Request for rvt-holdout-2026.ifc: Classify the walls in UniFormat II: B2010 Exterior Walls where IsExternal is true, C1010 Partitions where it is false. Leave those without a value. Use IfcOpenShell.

First a look at what the model holds.

```python
import ifcopenshell
import ifcopenshell.util.element

model = ifcopenshell.open("rvt-holdout-2026.ifc")
print(model.schema)
print("classifications:", [c.Name for c in model.by_type("IfcClassification")])
values = [ifcopenshell.util.element.get_pset(e, "Pset_WallCommon", "IsExternal") for e in model.by_type("IfcWall")]
for value in (True, False, None):
    print("IsExternal", value, values.count(value))
```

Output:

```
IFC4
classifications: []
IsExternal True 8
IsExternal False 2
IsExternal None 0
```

```python
import ifcopenshell
import ifcopenshell.api.classification
import ifcopenshell.util.element

model = ifcopenshell.open("rvt-holdout-2026.ifc")

system = ifcopenshell.api.classification.add_classification(model, classification="UniFormat II")

walls = model.by_type("IfcWall")
external = {e: ifcopenshell.util.element.get_pset(e, "Pset_WallCommon", "IsExternal") for e in walls}
for flag, code, name in ((True, "B2010", "Exterior Walls"), (False, "C1010", "Partitions")):
    products = [e for e in walls if external[e] is flag]
    ifcopenshell.api.classification.add_reference(
        model, products=products, classification=system, identification=code, name=name
    )
    print(code, len(products))

model.write("rvt-holdout-2026_edited.ifc")
```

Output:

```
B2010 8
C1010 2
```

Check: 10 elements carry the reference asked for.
